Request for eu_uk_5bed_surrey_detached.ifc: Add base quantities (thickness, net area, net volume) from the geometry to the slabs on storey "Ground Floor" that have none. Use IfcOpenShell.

First a look at what the model holds.

```python
import ifcopenshell
import ifcopenshell.util.element
import ifcopenshell.util.unit

model = ifcopenshell.open("eu_uk_5bed_surrey_detached.ifc")
print(model.schema)
for unit_type in ("LENGTHUNIT", "AREAUNIT", "VOLUMEUNIT"):
    print(unit_type, ifcopenshell.util.unit.calculate_unit_scale(model, unit_type))
storey = next(s for s in model.by_type("IfcBuildingStorey") if s.Name == "Ground Floor")
slabs = [e for e in ifcopenshell.util.element.get_decomposition(storey) if e.is_a("IfcSlab")]
for e in sorted(slabs, key=lambda e: e.id()):
    print(e.id(), e.is_a(), e.Name, list(ifcopenshell.util.element.get_psets(e, qtos_only=True)), sep=" | ")
```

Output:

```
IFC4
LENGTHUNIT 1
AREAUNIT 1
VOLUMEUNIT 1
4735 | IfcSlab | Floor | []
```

```python
import ifcopenshell
import ifcopenshell.api.pset
import ifcopenshell.geom
import ifcopenshell.util.element
import ifcopenshell.util.shape
import ifcopenshell.util.unit

model = ifcopenshell.open("eu_uk_5bed_surrey_detached.ifc")
unit_scale = ifcopenshell.util.unit.calculate_unit_scale(model)
area_scale = ifcopenshell.util.unit.calculate_unit_scale(model, "AREAUNIT")
volume_scale = ifcopenshell.util.unit.calculate_unit_scale(model, "VOLUMEUNIT")
settings = ifcopenshell.geom.settings()

storey = next(s for s in model.by_type("IfcBuildingStorey") if s.Name == "Ground Floor")
slabs = [e for e in ifcopenshell.util.element.get_decomposition(storey) if e.is_a("IfcSlab")]

for e in sorted(slabs, key=lambda e: e.id()):
    if ifcopenshell.util.element.get_psets(e, qtos_only=True, should_inherit=False):
        continue
    # Geometry comes back in metres, in the element's own axes.
    shape = ifcopenshell.geom.create_shape(settings, e)
    values = {
        "Width": ifcopenshell.util.shape.get_z(shape.geometry) / unit_scale,
        "NetArea": ifcopenshell.util.shape.get_footprint_area(shape.geometry) / area_scale,
        "NetVolume": ifcopenshell.util.shape.get_volume(shape.geometry) / volume_scale,
    }
    qto = ifcopenshell.api.pset.add_qto(model, product=e, name="Qto_SlabBaseQuantities")
    ifcopenshell.api.pset.edit_qto(model, qto=qto, properties=values)
    print(e.id(), {k: round(v, 3) for k, v in values.items()})

model.write("eu_uk_5bed_surrey_detached-out.ifc")
```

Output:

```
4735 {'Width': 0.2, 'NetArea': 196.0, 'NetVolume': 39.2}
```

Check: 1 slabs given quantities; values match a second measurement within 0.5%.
